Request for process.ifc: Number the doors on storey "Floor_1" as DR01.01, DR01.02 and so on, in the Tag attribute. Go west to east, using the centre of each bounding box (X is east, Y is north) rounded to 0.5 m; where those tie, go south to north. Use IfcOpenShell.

First a look at what the model holds.

```python
import ifcopenshell
import ifcopenshell.util.element
import ifcopenshell.util.placement

model = ifcopenshell.open("process.ifc")
print(model.schema)
storey = next(s for s in model.by_type("IfcBuildingStorey") if s.Name == "Floor_1")
doors = [e for e in ifcopenshell.util.element.get_decomposition(storey) if e.is_a("IfcDoor")]
for e in sorted(doors, key=lambda e: e.id()):
    origin = ifcopenshell.util.placement.get_local_placement(e.ObjectPlacement)[:3, 3]
    print(e.id(), e.Tag, e.Name, origin.round(2) + 0.0, sep=" | ")
```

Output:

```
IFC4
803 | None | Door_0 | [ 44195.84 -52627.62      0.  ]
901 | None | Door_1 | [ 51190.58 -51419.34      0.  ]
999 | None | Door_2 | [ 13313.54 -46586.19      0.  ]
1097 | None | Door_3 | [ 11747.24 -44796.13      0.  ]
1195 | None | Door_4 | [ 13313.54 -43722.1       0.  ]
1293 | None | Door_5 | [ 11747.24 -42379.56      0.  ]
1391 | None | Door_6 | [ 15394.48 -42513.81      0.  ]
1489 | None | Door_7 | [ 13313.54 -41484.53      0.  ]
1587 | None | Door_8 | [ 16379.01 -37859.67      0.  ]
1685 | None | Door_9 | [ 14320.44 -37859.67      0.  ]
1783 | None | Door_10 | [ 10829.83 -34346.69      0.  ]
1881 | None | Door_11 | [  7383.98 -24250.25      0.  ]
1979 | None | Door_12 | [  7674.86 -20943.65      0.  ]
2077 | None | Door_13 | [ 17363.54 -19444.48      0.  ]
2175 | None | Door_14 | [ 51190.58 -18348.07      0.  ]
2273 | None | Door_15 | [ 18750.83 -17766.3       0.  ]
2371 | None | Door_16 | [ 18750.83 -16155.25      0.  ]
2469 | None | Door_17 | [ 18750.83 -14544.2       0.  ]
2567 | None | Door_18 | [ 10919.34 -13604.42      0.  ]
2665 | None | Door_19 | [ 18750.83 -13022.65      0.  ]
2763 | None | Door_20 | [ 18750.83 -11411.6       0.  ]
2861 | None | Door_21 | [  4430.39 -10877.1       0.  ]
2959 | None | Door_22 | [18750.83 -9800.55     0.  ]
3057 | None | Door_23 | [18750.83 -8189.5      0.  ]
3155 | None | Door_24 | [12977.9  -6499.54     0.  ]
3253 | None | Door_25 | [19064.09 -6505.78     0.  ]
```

```python
import ifcopenshell
import ifcopenshell.geom
import ifcopenshell.util.element
import ifcopenshell.util.shape

model = ifcopenshell.open("process.ifc")
settings = ifcopenshell.geom.settings()
settings.set("use-world-coords", True)


def centre(element):
    shape = ifcopenshell.geom.create_shape(settings, element)
    return ifcopenshell.util.shape.get_bbox_centroid(shape.geometry)


storey = next(s for s in model.by_type("IfcBuildingStorey") if s.Name == "Floor_1")
doors = [e for e in ifcopenshell.util.element.get_decomposition(storey) if e.is_a("IfcDoor")]

# Insertion points can sit at a corner or the storey origin, so sort by the geometry (in metres).
centres = {e: centre(e) for e in doors}
doors.sort(key=lambda e: (round(centres[e][0] / 0.5), centres[e][1]))

for i, e in enumerate(doors, start=1):
    number = f"DR01.{i:02d}"
    e.Tag = number
    print(e.id(), number)

model.write("process-out.ifc")
```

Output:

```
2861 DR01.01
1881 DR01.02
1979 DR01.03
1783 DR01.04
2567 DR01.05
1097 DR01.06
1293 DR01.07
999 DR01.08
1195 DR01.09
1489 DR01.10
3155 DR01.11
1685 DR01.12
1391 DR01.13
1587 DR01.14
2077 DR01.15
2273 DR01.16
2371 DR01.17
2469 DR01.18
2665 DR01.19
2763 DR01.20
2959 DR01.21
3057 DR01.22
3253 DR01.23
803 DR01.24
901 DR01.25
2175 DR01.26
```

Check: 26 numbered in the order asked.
